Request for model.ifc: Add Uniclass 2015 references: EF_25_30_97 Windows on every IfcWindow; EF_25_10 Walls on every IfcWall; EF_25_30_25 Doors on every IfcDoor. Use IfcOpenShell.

First a look at what the model holds.

```python
import ifcopenshell

model = ifcopenshell.open("model.ifc")
print(model.schema)
print("classifications:", [c.Name for c in model.by_type("IfcClassification")])
for ifc_class in ("IfcDoor", "IfcRoof", "IfcStair", "IfcWall", "IfcWindow"):
    print(ifc_class, len(model.by_type(ifc_class)))
```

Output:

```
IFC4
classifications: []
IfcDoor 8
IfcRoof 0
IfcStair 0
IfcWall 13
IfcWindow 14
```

```python
import ifcopenshell
import ifcopenshell.api.classification

model = ifcopenshell.open("model.ifc")

system = ifcopenshell.api.classification.add_classification(model, classification="Uniclass 2015")

codes = {
    "IfcWindow": ("EF_25_30_97", "Windows"),
    "IfcWall": ("EF_25_10", "Walls"),
    "IfcDoor": ("EF_25_30_25", "Doors"),
}
for ifc_class, (code, name) in codes.items():
    products = model.by_type(ifc_class)
    ifcopenshell.api.classification.add_reference(
        model, products=products, classification=system, identification=code, name=name
    )
    print(code, len(products))

model.write("model_rev.ifc")
```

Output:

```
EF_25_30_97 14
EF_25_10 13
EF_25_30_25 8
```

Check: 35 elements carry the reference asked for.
